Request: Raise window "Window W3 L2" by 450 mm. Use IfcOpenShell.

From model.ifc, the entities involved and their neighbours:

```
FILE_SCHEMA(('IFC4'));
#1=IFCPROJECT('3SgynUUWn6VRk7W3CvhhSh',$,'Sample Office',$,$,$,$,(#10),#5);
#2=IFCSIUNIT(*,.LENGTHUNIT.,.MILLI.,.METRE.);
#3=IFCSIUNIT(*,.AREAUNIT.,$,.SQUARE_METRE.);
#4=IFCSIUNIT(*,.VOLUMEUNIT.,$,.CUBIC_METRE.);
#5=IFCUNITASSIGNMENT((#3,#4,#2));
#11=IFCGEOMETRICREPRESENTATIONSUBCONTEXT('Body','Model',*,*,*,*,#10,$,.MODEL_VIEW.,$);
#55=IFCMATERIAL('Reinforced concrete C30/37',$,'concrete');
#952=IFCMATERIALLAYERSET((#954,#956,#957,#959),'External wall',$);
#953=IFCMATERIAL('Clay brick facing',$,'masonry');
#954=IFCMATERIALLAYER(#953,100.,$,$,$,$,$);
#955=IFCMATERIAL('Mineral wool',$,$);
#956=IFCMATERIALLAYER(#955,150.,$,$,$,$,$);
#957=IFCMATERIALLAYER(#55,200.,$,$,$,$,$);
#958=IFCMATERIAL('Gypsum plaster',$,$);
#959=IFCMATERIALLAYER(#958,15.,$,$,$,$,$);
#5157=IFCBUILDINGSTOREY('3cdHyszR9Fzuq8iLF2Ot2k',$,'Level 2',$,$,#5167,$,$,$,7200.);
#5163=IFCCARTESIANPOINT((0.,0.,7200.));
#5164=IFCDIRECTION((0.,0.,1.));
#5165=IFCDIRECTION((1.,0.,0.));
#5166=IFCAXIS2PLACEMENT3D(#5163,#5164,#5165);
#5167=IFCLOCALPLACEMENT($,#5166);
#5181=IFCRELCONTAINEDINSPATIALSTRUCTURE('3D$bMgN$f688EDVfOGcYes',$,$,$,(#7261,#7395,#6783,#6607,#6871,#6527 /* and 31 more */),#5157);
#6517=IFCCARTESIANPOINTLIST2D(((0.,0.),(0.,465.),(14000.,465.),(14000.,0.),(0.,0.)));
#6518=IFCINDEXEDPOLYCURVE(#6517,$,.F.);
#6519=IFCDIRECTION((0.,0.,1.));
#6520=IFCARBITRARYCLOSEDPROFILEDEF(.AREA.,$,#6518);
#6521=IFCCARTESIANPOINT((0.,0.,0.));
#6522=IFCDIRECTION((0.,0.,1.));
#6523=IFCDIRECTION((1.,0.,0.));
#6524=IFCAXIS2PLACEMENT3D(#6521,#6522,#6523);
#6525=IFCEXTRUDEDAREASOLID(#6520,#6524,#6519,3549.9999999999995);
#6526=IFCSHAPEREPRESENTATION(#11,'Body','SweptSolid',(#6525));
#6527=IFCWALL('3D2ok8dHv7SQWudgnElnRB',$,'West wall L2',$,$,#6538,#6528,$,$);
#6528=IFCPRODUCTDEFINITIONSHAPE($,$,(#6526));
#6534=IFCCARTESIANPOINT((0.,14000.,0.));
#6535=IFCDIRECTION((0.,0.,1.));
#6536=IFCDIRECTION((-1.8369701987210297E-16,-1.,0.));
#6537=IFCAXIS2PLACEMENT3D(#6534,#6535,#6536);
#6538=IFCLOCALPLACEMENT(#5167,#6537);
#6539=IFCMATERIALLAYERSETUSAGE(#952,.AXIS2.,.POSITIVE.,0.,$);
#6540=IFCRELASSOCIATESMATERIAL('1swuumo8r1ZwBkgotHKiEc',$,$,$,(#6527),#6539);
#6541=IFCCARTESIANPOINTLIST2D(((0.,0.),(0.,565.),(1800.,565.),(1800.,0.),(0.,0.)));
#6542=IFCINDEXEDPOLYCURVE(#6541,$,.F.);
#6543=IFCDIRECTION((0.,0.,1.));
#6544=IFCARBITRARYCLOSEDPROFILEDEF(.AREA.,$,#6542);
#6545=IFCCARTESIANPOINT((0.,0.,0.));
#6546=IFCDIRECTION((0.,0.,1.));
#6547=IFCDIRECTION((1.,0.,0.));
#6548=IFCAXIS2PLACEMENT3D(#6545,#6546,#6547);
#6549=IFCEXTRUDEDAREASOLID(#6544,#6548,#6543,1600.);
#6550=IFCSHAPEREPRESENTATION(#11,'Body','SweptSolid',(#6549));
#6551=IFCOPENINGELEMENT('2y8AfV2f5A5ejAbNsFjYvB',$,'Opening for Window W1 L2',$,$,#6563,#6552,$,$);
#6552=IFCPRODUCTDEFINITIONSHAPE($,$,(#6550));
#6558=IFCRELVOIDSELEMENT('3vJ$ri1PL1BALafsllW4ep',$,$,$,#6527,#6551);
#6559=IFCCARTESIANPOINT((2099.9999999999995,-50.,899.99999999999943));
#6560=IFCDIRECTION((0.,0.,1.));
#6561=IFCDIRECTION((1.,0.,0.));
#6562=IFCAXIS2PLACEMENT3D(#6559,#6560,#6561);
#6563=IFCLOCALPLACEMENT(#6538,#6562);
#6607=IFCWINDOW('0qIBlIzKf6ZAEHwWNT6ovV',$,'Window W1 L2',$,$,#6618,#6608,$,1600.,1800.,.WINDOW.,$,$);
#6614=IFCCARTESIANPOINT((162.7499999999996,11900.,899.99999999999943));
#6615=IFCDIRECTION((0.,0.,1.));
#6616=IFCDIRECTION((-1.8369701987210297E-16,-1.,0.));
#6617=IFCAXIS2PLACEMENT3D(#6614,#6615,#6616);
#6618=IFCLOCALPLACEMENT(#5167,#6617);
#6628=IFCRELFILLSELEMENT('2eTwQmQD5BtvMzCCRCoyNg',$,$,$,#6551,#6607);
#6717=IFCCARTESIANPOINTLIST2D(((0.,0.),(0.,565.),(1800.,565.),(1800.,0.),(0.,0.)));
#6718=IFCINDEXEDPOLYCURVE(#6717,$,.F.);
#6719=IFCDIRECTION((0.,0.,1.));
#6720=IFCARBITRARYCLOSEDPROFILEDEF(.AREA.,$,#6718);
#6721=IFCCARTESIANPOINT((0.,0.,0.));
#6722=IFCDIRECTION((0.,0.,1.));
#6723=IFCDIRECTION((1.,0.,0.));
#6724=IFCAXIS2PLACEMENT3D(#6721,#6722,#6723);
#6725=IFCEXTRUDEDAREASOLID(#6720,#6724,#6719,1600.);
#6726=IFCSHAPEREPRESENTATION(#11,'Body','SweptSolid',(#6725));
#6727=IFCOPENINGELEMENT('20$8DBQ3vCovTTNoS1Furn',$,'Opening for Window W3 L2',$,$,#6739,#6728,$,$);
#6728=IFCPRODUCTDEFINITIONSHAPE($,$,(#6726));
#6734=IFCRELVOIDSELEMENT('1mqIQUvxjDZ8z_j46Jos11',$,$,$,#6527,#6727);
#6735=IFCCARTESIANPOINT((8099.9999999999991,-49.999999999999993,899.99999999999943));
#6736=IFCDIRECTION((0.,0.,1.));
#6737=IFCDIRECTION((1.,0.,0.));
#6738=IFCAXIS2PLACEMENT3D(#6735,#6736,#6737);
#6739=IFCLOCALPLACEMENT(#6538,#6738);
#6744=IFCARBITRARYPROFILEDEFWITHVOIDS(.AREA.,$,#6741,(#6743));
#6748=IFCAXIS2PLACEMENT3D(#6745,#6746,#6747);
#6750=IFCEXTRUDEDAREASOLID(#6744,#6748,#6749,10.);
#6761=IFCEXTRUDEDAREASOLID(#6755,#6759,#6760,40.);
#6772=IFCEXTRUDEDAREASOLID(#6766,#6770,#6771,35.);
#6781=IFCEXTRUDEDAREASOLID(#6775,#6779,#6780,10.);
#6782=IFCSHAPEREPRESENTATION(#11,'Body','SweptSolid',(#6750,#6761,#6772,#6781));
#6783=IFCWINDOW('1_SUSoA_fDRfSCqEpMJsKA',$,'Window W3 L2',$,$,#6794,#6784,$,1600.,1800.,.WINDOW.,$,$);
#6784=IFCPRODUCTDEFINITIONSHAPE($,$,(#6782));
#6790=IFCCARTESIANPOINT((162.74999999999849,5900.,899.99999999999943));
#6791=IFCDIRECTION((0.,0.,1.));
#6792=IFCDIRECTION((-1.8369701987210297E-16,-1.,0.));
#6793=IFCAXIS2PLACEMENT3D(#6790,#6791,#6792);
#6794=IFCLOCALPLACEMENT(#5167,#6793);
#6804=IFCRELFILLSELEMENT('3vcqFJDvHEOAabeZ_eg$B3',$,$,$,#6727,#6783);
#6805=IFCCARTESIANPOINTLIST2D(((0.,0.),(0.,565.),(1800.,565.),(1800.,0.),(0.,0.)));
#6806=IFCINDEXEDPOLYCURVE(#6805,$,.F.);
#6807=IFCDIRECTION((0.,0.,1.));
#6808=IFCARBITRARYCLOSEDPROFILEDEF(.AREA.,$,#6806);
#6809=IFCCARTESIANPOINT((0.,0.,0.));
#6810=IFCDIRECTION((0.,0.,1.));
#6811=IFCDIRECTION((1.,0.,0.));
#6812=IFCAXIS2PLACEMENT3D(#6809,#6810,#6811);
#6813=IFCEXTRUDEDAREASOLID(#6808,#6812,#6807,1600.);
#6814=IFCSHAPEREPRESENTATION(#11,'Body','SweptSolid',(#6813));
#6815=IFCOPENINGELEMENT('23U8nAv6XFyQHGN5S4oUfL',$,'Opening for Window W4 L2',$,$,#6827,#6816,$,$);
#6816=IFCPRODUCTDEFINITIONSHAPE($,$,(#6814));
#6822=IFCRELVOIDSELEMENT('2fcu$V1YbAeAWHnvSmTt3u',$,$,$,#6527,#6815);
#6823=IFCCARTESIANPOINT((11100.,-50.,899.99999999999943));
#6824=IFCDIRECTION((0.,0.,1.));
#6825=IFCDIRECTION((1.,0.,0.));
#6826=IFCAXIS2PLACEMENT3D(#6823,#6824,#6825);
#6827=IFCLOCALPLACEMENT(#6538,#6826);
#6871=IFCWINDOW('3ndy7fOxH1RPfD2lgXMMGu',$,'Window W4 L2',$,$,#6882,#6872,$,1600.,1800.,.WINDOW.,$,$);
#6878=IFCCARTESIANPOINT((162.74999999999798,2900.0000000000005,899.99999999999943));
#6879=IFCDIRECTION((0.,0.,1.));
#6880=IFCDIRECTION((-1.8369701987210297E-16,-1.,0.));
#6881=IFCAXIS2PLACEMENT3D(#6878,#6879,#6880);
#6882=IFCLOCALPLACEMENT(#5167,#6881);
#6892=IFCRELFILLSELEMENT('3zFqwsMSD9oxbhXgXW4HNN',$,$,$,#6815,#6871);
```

```python
import numpy as np
import ifcopenshell
import ifcopenshell.api.geometry
import ifcopenshell.util.placement
import ifcopenshell.util.unit

model = ifcopenshell.open("model.ifc")
unit_scale = ifcopenshell.util.unit.calculate_unit_scale(model)

window = model.by_guid("1_SUSoA_fDRfSCqEpMJsKA")
opening = window.FillsVoids[0].RelatingOpeningElement
dz = 0.45 / unit_scale

shift = np.array([0.0, 0.0, dz])
# The window is not placed relative to its opening, so move both.
for product in (opening, window):
    matrix = ifcopenshell.util.placement.get_local_placement(product.ObjectPlacement)
    matrix[:3, 3] += shift
    ifcopenshell.api.geometry.edit_object_placement(model, product=product, matrix=matrix, is_si=False)

print(f"moved by {dz * unit_scale:+.3f} m")

model.write("model_rev.ifc")
```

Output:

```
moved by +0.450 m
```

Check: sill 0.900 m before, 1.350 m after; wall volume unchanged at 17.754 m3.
